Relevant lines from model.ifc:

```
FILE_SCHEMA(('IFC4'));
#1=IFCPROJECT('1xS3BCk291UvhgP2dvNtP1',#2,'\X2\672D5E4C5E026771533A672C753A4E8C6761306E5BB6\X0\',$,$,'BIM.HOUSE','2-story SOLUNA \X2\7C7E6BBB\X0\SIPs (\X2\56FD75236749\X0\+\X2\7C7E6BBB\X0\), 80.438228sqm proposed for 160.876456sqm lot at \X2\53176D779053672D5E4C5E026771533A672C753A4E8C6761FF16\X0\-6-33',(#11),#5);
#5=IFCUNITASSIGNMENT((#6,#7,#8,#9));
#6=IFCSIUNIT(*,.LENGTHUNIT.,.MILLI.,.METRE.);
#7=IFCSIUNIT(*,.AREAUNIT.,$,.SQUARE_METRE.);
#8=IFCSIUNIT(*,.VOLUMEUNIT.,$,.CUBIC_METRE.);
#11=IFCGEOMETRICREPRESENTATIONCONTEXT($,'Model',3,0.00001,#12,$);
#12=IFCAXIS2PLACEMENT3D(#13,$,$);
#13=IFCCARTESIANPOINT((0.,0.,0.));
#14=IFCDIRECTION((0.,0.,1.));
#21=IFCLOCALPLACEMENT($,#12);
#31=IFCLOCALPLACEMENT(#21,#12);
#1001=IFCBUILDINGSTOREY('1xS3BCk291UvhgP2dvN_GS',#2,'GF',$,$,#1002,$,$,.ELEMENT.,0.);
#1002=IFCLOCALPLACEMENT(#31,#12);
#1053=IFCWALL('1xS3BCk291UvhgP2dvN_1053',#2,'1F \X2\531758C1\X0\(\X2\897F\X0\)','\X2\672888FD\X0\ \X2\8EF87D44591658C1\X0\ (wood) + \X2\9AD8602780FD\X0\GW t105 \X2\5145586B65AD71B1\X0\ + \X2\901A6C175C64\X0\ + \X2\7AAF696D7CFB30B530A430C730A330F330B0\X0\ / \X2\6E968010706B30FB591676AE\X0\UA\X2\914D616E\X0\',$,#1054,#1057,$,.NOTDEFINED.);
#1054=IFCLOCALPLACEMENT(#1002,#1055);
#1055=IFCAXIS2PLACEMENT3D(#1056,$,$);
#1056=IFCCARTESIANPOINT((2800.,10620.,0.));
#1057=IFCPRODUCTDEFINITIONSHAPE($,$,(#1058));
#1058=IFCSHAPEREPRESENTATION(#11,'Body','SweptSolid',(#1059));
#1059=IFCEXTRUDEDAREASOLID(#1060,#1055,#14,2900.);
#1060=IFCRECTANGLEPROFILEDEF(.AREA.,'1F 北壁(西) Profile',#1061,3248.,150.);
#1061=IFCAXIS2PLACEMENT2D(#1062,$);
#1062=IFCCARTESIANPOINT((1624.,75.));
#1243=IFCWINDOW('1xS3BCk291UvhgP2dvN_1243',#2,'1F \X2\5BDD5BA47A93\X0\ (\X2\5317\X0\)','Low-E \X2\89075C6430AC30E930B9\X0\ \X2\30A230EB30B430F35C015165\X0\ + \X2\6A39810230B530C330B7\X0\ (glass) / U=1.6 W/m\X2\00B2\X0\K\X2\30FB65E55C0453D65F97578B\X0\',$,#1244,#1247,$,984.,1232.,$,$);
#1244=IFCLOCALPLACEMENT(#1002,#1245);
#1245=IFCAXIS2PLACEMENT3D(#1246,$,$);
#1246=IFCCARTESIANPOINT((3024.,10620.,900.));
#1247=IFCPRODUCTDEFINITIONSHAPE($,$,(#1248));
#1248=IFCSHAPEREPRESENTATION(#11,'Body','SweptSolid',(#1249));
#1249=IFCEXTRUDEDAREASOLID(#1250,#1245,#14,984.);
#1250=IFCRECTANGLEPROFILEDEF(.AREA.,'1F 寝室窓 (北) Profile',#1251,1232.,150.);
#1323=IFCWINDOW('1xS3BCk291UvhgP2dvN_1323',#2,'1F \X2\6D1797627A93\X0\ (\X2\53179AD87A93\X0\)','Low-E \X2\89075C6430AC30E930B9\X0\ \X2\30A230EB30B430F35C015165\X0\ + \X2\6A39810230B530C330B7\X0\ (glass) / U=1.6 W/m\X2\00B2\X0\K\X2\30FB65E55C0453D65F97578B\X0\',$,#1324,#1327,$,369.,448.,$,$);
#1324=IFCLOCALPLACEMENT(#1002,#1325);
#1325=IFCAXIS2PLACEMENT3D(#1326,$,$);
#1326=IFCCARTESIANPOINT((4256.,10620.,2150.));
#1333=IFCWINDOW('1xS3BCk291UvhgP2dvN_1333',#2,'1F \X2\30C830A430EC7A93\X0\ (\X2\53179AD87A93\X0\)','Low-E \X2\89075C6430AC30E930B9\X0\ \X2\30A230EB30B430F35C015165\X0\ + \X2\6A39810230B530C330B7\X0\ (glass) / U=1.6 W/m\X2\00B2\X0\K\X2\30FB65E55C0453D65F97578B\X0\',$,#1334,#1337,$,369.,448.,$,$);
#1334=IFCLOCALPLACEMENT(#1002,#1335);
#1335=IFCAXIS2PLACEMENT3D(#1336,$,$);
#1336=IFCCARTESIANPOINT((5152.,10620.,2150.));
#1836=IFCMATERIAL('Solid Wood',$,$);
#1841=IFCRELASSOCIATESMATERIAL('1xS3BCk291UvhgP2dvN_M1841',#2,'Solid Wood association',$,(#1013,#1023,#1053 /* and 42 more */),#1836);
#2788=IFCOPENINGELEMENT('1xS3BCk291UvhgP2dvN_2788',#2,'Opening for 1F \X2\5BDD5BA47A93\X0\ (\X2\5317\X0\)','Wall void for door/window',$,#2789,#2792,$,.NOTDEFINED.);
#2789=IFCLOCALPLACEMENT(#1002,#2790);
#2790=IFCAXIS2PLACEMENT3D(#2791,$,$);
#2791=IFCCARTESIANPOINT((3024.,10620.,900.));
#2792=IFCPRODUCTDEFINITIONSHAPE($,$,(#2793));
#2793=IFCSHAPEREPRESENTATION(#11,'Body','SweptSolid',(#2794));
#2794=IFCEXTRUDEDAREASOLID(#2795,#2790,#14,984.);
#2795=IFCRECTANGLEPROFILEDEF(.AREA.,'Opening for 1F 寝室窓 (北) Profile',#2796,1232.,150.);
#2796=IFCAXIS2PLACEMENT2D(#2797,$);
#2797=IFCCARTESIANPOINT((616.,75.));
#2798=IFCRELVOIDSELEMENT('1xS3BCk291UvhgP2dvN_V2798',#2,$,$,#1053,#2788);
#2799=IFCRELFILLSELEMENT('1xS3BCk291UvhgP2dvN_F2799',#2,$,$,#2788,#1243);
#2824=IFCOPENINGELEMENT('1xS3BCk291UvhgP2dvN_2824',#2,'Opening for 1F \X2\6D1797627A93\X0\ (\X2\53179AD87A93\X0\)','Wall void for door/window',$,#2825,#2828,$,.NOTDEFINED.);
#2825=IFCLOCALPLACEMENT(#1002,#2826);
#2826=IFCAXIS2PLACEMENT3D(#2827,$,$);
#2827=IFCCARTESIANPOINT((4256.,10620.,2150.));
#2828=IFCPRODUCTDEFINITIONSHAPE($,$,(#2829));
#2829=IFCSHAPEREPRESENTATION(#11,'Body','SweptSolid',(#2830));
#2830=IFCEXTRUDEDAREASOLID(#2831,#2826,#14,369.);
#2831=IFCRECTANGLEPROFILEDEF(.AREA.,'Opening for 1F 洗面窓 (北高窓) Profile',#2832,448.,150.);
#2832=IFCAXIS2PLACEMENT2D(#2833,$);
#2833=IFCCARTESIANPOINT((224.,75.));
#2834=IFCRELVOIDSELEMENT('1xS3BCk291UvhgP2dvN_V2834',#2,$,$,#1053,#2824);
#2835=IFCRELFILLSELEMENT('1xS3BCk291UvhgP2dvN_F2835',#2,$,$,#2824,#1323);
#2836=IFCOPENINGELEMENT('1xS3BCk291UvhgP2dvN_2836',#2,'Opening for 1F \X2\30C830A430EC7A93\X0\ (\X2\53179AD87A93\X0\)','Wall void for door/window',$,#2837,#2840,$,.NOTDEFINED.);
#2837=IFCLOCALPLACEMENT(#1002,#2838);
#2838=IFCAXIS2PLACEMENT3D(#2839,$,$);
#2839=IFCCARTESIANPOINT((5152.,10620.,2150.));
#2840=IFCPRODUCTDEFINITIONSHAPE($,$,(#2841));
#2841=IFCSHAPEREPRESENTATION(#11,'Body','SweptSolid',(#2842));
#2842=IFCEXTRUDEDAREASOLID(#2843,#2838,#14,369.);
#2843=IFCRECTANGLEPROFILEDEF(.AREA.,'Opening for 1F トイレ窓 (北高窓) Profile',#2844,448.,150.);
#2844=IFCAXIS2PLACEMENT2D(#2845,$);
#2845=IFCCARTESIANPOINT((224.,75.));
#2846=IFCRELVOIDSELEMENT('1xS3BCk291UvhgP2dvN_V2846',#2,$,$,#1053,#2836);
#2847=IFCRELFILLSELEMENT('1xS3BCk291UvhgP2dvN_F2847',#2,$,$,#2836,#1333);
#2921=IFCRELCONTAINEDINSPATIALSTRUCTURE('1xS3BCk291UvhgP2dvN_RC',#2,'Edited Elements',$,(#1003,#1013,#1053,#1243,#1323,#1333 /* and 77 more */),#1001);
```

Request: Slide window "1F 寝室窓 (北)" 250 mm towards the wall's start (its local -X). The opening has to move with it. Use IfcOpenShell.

```python
import ifcopenshell
import ifcopenshell.api.geometry
import ifcopenshell.util.placement

model = ifcopenshell.open("model.ifc")

window = model.by_guid("1xS3BCk291UvhgP2dvN_1243")
opening = window.FillsVoids[0].RelatingOpeningElement
wall = opening.VoidsElements[0].RelatingBuildingElement

wall_matrix = ifcopenshell.util.placement.get_local_placement(wall.ObjectPlacement)
shift = wall_matrix[:3, 0] * -250.0
before = ifcopenshell.util.placement.get_local_placement(window.ObjectPlacement)[:3, 3].copy()

# The window is not placed relative to its opening, so move both.
for product in (opening, window):
    matrix = ifcopenshell.util.placement.get_local_placement(product.ObjectPlacement)
    matrix[:3, 3] += shift
    ifcopenshell.api.geometry.edit_object_placement(model, product=product, matrix=matrix, is_si=False)

after = ifcopenshell.util.placement.get_local_placement(window.ObjectPlacement)[:3, 3]
print("window moved by", (after - before).round(3) + 0.0)

model.write("model-out.ifc")
```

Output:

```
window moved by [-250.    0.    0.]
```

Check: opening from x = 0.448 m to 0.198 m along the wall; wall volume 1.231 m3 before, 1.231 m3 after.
